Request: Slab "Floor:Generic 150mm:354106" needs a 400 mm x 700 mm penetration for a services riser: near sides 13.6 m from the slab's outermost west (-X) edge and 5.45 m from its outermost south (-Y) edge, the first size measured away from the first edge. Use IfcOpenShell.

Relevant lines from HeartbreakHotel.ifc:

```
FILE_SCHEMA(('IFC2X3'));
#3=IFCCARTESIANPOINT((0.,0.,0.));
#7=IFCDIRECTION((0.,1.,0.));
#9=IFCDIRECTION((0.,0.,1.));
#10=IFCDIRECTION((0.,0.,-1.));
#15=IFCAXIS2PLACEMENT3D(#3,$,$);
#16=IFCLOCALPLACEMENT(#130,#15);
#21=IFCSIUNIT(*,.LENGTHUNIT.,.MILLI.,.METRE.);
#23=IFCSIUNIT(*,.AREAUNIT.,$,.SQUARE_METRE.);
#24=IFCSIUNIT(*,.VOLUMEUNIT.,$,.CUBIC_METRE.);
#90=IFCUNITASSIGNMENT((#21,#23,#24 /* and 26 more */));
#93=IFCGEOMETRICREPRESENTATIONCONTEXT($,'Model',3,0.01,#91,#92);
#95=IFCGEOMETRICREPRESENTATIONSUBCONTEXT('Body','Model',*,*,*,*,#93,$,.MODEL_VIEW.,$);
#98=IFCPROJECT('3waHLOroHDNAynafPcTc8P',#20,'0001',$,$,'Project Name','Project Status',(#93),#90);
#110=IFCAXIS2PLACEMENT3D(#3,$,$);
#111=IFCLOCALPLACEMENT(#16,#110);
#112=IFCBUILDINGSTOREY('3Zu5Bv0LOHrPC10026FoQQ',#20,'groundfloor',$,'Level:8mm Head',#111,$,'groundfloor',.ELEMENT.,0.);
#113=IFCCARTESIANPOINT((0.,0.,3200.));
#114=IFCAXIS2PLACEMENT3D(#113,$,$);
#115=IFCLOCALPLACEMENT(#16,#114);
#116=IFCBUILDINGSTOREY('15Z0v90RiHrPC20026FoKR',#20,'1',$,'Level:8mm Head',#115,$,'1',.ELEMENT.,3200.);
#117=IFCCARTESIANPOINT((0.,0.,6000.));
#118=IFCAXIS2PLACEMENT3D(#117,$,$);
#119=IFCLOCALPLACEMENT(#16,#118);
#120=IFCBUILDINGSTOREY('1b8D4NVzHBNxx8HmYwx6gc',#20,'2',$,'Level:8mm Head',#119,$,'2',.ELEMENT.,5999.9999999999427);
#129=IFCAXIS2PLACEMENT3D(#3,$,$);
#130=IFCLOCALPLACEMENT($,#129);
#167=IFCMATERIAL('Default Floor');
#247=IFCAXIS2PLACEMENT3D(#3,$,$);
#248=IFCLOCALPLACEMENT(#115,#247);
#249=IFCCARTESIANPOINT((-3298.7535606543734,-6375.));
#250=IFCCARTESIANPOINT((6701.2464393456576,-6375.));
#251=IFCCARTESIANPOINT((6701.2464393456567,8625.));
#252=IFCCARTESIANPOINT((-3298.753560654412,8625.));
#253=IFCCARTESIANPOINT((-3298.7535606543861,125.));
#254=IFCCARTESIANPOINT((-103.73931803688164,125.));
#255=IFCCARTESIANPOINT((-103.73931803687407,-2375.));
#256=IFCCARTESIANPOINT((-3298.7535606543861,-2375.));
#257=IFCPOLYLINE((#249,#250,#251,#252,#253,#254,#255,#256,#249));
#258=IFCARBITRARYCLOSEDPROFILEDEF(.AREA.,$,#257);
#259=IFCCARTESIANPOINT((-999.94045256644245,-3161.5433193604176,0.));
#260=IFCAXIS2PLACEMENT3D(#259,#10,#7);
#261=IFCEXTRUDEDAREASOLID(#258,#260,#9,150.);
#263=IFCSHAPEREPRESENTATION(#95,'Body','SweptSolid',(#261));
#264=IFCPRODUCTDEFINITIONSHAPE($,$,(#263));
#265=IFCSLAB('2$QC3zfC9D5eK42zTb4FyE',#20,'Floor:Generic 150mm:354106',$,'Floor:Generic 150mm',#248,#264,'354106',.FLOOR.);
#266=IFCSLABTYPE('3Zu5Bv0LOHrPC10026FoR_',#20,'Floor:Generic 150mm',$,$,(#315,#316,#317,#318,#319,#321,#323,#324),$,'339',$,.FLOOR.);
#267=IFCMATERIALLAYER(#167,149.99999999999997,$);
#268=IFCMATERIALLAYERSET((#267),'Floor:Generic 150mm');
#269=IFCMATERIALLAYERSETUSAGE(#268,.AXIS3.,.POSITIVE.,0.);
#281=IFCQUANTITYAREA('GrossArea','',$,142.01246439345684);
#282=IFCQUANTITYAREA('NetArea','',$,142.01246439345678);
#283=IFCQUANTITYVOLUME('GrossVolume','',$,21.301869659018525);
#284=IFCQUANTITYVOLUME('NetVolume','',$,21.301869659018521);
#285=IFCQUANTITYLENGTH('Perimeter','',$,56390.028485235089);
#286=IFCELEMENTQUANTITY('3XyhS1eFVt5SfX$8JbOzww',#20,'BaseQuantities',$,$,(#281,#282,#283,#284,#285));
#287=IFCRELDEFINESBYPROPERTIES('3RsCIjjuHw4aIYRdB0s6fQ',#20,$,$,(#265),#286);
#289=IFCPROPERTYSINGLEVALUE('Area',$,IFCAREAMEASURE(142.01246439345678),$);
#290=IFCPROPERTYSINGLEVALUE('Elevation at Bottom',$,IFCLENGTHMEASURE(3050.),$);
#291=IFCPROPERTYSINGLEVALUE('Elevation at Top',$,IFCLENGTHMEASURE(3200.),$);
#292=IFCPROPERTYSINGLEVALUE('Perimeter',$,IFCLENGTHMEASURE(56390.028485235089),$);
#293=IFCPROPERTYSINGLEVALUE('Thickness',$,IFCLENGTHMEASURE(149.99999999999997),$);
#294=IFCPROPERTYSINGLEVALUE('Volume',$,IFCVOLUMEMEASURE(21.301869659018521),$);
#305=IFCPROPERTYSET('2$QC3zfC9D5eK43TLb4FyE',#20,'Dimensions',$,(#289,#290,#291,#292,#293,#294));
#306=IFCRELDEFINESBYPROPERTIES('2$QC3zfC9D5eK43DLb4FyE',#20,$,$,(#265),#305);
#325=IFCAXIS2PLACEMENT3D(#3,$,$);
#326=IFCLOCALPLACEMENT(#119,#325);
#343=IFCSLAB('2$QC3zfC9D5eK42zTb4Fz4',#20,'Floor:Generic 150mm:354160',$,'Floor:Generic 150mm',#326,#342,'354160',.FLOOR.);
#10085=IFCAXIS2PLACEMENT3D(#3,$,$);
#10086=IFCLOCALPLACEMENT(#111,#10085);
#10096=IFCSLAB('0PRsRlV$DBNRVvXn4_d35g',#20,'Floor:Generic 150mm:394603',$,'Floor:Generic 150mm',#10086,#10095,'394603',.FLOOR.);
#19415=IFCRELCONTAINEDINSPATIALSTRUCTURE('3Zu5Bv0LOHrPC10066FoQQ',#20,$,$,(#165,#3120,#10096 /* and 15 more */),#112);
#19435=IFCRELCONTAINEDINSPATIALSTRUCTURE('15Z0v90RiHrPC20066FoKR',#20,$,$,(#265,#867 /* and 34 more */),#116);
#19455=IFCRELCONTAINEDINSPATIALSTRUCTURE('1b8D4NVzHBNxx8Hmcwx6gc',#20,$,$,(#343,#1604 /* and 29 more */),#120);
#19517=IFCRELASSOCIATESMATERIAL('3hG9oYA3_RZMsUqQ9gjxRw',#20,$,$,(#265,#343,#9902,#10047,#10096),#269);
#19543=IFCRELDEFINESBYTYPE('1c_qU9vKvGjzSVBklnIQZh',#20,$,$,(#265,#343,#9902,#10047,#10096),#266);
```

```python
import numpy as np
import ifcopenshell
import ifcopenshell.api.feature
import ifcopenshell.api.geometry
import ifcopenshell.api.pset
import ifcopenshell.api.root
import ifcopenshell.geom
import ifcopenshell.util.element
import ifcopenshell.util.placement
import ifcopenshell.util.representation
import ifcopenshell.util.shape
import ifcopenshell.util.unit

model = ifcopenshell.open("HeartbreakHotel.ifc")
unit_scale = ifcopenshell.util.unit.calculate_unit_scale(model)
area_scale = ifcopenshell.util.unit.calculate_unit_scale(model, "AREAUNIT")
volume_scale = ifcopenshell.util.unit.calculate_unit_scale(model, "VOLUMEUNIT")
settings = ifcopenshell.geom.settings()


def volume(element):
    """Net volume in cubic metres, openings subtracted."""
    shape = ifcopenshell.geom.create_shape(settings, element)
    return ifcopenshell.util.shape.get_volume(shape.geometry)


slab = model.by_guid("2$QC3zfC9D5eK42zTb4FyE")
before = volume(slab)

# Extent in the slab's own axes, in metres. The edges named are its -X and -Y sides.
slab_shape = ifcopenshell.geom.create_shape(settings, slab)
vertices = ifcopenshell.util.shape.get_vertices(slab_shape.geometry)
x_min, y_min, bottom = vertices.min(axis=0)
top = vertices[:, 2].max()

opening = ifcopenshell.api.root.create_entity(model, ifc_class="IfcOpeningElement", name="Services riser opening")
context = ifcopenshell.util.representation.get_context(model, "Model", "Body", "MODEL_VIEW")
width, depth = 0.4, 0.7
outline = [(0.0, 0.0), (width, 0.0), (width, depth), (0.0, depth), (0.0, 0.0)]
# Overshoot both faces by 50 mm so the cut is clean.
shape = ifcopenshell.api.geometry.add_slab_representation(
    model, context=context, depth=top - bottom + 0.1, polyline=outline
)
ifcopenshell.api.geometry.assign_representation(model, product=opening, representation=shape)

matrix = ifcopenshell.util.placement.get_local_placement(slab.ObjectPlacement)
matrix[:, 3] = matrix @ np.append(np.array([x_min + 13.6, y_min + 5.45, bottom - 0.05]) / unit_scale, 1.0)
ifcopenshell.api.geometry.edit_object_placement(model, product=opening, matrix=matrix, is_si=False)
ifcopenshell.api.feature.add_feature(model, feature=opening, element=slab)

after = volume(slab)

# Update the slab's stored quantities.
qto = model.by_id(ifcopenshell.util.element.get_pset(slab, "BaseQuantities", should_inherit=False)["id"])
ifcopenshell.api.pset.edit_qto(model, qto=qto, properties={
    "NetArea": after / (top - bottom) / area_scale,
    "NetVolume": after / volume_scale,
})
pset = model.by_id(ifcopenshell.util.element.get_pset(slab, "Dimensions", should_inherit=False)["id"])
ifcopenshell.api.pset.edit_pset(model, pset=pset, properties={
    "Area": model.create_entity("IfcAreaMeasure", after / (top - bottom) / area_scale),
    "Volume": model.create_entity("IfcVolumeMeasure", after / volume_scale),
})

print(f"slab volume {before:.3f} -> {after:.3f} m3")

model.write("HeartbreakHotel_updated.ifc")
```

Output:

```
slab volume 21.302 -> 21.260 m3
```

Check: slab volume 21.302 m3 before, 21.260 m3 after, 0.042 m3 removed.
